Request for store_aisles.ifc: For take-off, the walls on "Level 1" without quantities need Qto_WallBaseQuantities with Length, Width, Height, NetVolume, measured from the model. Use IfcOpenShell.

First a look at what the model holds.

```python
import ifcopenshell
import ifcopenshell.util.element
import ifcopenshell.util.unit

model = ifcopenshell.open("store_aisles.ifc")
print(model.schema)
for unit_type in ("LENGTHUNIT", "AREAUNIT", "VOLUMEUNIT"):
    print(unit_type, ifcopenshell.util.unit.calculate_unit_scale(model, unit_type))
storey = next(s for s in model.by_type("IfcBuildingStorey") if s.Name == "Level 1")
walls = [e for e in ifcopenshell.util.element.get_decomposition(storey) if e.is_a("IfcWall")]
for e in sorted(walls, key=lambda e: e.id()):
    print(e.id(), e.is_a(), e.Name, list(ifcopenshell.util.element.get_psets(e, qtos_only=True)), sep=" | ")
```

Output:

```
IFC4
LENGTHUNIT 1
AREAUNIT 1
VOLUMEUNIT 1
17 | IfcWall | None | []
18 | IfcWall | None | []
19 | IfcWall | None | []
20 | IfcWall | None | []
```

```python
import ifcopenshell
import ifcopenshell.api.pset
import ifcopenshell.geom
import ifcopenshell.util.element
import ifcopenshell.util.shape
import ifcopenshell.util.unit

model = ifcopenshell.open("store_aisles.ifc")
unit_scale = ifcopenshell.util.unit.calculate_unit_scale(model)
volume_scale = ifcopenshell.util.unit.calculate_unit_scale(model, "VOLUMEUNIT")
settings = ifcopenshell.geom.settings()

storey = next(s for s in model.by_type("IfcBuildingStorey") if s.Name == "Level 1")
walls = [e for e in ifcopenshell.util.element.get_decomposition(storey) if e.is_a("IfcWall")]

for e in sorted(walls, key=lambda e: e.id()):
    if ifcopenshell.util.element.get_psets(e, qtos_only=True, should_inherit=False):
        continue
    # Geometry comes back in metres, in the element's own axes.
    shape = ifcopenshell.geom.create_shape(settings, e)
    values = {
        "Length": ifcopenshell.util.shape.get_x(shape.geometry) / unit_scale,
        "Width": ifcopenshell.util.shape.get_y(shape.geometry) / unit_scale,
        "Height": ifcopenshell.util.shape.get_z(shape.geometry) / unit_scale,
        "NetVolume": ifcopenshell.util.shape.get_volume(shape.geometry) / volume_scale,
    }
    qto = ifcopenshell.api.pset.add_qto(model, product=e, name="Qto_WallBaseQuantities")
    ifcopenshell.api.pset.edit_qto(model, qto=qto, properties=values)
    print(e.id(), {k: round(v, 3) for k, v in values.items()})

model.write("store_aisles_updated.ifc")
```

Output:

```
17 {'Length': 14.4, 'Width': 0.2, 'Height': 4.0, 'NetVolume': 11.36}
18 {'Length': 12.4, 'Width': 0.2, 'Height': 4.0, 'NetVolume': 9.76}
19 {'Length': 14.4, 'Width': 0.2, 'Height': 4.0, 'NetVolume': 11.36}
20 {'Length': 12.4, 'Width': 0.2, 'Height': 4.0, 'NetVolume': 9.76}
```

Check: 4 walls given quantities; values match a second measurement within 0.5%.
